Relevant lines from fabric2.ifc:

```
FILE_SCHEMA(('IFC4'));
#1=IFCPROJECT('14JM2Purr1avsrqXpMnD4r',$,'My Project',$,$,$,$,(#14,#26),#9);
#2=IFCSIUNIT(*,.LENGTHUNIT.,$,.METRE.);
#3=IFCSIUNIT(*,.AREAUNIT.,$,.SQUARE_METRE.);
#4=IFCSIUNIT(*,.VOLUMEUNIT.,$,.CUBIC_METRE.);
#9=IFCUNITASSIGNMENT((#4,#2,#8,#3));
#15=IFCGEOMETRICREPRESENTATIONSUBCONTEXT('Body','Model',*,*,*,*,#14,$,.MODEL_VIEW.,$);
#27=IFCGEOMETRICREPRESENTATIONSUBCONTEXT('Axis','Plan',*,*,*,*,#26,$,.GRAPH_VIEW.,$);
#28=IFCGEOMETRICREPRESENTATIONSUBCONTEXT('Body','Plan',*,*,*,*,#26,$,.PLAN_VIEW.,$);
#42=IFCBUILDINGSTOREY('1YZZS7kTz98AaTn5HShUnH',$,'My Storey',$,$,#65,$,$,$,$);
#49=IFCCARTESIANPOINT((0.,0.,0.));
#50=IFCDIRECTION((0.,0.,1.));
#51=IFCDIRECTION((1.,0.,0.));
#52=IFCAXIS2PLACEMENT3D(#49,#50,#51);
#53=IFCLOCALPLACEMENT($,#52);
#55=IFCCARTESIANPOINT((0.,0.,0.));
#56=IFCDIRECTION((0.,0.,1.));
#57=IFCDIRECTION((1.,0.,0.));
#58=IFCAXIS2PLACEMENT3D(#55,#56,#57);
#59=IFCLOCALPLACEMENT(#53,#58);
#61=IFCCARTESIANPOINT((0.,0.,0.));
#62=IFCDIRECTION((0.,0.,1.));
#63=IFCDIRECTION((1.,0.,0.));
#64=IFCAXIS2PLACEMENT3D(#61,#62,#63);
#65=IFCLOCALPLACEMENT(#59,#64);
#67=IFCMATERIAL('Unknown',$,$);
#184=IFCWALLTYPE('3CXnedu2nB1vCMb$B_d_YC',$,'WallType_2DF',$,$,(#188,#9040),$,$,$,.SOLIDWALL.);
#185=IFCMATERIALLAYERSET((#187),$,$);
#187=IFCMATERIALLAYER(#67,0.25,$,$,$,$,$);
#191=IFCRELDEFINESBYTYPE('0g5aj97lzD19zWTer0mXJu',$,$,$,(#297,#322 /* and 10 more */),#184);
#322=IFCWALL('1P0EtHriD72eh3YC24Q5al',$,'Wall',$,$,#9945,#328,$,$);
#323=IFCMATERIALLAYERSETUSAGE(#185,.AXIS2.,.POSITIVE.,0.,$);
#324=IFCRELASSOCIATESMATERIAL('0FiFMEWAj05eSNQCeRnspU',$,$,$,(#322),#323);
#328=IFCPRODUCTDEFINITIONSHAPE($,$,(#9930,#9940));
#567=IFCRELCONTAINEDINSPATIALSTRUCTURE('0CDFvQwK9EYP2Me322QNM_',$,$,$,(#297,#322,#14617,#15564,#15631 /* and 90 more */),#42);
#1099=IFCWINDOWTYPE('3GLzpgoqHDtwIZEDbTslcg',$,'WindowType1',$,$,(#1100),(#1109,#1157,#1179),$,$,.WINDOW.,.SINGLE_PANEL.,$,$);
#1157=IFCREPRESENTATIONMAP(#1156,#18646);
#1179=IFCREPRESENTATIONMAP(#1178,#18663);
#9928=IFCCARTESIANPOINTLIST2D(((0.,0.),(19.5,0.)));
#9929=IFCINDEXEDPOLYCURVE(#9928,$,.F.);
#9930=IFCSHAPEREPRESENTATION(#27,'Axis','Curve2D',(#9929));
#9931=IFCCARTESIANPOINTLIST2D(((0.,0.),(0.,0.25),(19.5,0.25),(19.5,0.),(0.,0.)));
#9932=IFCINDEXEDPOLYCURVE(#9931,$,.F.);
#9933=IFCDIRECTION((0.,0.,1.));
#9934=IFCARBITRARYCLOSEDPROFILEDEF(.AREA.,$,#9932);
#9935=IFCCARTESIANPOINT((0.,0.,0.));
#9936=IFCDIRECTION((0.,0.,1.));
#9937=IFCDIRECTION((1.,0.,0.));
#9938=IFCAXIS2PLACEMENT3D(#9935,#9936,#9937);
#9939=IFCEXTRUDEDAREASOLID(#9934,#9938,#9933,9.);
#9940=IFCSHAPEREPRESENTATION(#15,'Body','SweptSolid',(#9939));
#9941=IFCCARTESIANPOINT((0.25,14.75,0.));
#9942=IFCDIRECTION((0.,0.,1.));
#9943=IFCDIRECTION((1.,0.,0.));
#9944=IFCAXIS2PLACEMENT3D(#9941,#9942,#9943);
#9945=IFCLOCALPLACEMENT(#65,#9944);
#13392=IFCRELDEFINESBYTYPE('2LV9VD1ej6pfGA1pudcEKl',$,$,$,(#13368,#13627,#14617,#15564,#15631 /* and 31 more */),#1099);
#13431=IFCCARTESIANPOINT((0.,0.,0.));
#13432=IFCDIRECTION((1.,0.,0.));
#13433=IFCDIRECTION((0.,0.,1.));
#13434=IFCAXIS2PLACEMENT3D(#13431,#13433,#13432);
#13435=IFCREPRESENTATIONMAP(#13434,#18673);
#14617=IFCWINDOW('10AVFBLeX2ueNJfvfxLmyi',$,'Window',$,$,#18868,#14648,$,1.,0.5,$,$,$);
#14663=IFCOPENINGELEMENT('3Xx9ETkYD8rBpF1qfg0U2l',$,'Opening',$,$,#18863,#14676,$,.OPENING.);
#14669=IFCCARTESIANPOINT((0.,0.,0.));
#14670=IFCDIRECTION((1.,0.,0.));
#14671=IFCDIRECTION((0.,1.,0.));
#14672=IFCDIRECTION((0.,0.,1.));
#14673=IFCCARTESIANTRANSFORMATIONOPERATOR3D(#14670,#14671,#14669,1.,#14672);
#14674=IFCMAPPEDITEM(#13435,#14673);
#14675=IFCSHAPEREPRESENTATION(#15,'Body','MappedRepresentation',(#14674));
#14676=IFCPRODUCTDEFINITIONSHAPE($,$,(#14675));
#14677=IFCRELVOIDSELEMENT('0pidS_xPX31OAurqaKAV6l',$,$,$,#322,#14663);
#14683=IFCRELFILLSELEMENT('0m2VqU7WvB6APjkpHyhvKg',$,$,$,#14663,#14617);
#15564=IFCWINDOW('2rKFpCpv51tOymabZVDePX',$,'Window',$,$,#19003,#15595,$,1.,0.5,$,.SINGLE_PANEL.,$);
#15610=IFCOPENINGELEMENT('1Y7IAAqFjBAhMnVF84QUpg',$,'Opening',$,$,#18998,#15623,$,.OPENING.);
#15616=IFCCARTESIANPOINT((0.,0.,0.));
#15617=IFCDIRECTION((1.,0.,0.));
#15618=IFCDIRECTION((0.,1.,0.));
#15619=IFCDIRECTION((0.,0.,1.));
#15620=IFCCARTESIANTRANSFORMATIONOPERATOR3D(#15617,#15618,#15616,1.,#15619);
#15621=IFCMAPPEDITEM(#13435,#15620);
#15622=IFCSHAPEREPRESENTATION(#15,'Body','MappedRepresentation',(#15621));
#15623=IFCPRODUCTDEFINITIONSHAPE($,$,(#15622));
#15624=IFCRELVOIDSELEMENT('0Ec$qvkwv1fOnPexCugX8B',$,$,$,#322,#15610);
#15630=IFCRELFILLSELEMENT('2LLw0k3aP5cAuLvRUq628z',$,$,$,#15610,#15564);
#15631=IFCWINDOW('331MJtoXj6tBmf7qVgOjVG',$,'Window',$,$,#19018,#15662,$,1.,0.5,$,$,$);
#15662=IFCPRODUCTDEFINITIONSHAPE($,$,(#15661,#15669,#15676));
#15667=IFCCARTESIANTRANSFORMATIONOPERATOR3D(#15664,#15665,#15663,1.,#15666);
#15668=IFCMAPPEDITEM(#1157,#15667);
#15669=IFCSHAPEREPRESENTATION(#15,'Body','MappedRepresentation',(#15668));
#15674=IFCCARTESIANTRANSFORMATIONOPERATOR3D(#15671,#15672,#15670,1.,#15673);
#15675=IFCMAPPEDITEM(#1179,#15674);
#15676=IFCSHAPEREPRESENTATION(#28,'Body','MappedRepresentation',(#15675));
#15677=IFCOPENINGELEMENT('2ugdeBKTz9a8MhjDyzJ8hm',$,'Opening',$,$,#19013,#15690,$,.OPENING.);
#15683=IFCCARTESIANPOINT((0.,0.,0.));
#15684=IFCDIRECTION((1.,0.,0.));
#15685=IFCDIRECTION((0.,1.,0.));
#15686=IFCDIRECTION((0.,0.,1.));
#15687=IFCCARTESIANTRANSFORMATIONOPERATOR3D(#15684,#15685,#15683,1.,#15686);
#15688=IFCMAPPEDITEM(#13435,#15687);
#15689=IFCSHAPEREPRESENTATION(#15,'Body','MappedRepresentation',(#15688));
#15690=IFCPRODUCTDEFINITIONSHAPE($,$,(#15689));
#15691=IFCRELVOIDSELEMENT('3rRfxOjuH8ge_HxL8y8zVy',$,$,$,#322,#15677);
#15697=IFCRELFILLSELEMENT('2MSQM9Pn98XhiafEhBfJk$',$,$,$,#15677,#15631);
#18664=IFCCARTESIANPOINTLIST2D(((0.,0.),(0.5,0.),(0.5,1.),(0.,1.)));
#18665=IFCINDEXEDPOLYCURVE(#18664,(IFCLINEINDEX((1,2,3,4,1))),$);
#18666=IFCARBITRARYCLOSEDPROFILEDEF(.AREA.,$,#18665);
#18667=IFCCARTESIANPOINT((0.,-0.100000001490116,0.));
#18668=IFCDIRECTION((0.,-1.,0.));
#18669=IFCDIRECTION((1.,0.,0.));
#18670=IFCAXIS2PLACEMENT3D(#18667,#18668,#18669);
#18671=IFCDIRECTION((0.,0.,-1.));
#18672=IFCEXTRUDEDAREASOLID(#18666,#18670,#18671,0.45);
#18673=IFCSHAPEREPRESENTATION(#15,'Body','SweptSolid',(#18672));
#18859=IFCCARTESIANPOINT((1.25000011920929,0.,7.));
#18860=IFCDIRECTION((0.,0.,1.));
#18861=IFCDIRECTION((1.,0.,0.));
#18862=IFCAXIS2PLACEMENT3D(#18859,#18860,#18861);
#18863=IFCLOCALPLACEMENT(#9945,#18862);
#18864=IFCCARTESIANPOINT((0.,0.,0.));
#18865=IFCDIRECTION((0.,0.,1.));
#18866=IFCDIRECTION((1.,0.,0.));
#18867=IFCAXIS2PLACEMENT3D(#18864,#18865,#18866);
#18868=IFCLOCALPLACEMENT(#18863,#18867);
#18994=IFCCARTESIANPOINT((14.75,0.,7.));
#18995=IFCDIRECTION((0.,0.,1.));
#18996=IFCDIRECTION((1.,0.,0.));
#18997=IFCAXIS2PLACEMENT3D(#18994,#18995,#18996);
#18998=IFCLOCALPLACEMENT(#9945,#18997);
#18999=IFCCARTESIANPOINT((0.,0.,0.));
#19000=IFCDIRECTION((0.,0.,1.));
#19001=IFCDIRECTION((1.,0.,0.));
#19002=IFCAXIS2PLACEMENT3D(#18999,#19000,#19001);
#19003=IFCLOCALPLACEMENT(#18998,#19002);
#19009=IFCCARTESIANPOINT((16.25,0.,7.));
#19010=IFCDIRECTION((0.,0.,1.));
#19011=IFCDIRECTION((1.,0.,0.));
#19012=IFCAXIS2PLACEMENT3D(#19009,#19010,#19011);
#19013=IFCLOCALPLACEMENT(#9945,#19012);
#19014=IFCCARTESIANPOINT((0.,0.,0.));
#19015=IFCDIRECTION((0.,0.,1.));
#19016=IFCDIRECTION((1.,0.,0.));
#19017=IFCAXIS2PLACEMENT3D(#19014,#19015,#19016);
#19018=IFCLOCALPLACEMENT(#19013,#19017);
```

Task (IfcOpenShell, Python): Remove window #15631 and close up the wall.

```python
import ifcopenshell
import ifcopenshell.api.feature
import ifcopenshell.api.root
import ifcopenshell.geom
import ifcopenshell.util.shape

model = ifcopenshell.open("fabric2.ifc")
settings = ifcopenshell.geom.settings()


def volume(element):
    """Net volume in cubic metres, openings subtracted."""
    shape = ifcopenshell.geom.create_shape(settings, element)
    return ifcopenshell.util.shape.get_volume(shape.geometry)


window = model.by_guid("331MJtoXj6tBmf7qVgOjVG")
opening = window.FillsVoids[0].RelatingOpeningElement
wall = opening.VoidsElements[0].RelatingBuildingElement
before = volume(wall)

ifcopenshell.api.root.remove_product(model, product=window)
ifcopenshell.api.feature.remove_feature(model, feature=opening)

after = volume(wall)

print(f"wall volume {before:.3f} -> {after:.3f} m3")

model.write("fabric2_rev.ifc")
```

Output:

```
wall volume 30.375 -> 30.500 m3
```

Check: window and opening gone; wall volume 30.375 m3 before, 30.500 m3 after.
